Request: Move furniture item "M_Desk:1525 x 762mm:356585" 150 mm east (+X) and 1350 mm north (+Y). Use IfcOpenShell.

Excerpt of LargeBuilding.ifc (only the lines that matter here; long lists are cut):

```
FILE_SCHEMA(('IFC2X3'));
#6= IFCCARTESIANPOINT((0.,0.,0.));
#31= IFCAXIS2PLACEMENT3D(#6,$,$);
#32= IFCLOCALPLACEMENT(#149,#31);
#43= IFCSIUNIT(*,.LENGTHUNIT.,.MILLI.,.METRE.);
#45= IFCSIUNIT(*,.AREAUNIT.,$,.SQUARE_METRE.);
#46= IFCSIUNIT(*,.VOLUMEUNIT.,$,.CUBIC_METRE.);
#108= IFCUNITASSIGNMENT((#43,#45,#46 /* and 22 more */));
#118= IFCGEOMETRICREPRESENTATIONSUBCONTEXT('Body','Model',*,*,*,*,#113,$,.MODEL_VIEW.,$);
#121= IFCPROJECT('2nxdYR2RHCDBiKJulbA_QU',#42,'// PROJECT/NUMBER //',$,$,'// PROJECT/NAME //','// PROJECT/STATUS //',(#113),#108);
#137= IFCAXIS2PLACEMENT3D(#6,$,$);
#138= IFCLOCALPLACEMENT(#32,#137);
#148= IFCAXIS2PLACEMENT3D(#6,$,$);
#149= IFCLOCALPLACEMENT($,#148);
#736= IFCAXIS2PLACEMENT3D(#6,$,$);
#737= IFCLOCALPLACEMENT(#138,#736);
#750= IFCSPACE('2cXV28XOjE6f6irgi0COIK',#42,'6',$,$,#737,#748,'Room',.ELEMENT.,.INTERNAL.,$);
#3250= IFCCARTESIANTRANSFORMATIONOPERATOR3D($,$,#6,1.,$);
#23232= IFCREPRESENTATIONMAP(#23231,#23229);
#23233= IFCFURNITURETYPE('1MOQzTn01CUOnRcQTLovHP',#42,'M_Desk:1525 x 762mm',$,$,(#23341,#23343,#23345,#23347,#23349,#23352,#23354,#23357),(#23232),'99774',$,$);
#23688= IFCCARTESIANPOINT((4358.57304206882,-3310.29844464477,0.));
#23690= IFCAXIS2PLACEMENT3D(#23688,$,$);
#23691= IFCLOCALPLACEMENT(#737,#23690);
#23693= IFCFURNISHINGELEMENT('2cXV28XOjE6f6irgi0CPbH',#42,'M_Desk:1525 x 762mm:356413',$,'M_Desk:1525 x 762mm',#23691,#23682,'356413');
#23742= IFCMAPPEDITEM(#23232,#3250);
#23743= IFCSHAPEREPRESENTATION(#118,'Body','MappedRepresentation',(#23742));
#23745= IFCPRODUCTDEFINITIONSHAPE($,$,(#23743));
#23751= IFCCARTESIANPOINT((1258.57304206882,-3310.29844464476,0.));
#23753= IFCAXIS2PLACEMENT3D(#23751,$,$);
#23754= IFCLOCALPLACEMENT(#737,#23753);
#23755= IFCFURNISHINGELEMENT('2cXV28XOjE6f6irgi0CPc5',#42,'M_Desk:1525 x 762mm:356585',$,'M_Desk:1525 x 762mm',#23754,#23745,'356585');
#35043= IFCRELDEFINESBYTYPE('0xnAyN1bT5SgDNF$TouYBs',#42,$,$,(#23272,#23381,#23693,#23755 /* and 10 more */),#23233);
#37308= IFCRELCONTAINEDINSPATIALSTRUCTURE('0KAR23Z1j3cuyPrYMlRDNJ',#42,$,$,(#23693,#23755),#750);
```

```python
import ifcopenshell
import ifcopenshell.api.geometry
import ifcopenshell.util.placement

model = ifcopenshell.open("LargeBuilding.ifc")

item = model.by_id(23755)
matrix = ifcopenshell.util.placement.get_local_placement(item.ObjectPlacement)
matrix[0, 3] += 150.0
matrix[1, 3] += 1350.0
ifcopenshell.api.geometry.edit_object_placement(model, product=item, matrix=matrix, is_si=False)

print(ifcopenshell.util.placement.get_local_placement(item.ObjectPlacement).round(3) + 0.0)

model.write("LargeBuilding_v2.ifc")
```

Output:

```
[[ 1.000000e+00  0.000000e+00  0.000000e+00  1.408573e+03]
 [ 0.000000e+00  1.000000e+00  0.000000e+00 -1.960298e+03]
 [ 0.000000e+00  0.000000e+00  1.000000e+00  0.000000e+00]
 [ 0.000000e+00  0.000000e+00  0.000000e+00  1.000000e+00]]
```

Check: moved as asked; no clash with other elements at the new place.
